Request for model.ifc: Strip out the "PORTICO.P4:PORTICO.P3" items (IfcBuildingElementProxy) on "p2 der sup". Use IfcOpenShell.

First a look at what the model holds.

```python
import ifcopenshell
import ifcopenshell.util.element

model = ifcopenshell.open("model.ifc")
print(model.schema)
storey = next(s for s in model.by_type("IfcBuildingStorey") if s.Name == "p2 der sup")
proxies = [e for e in ifcopenshell.util.element.get_decomposition(storey) if e.is_a("IfcBuildingElementProxy")]
seen = {}
for e in proxies:
    element_type = ifcopenshell.util.element.get_type(e)
    name = element_type.Name if element_type not in (None, e) else None
    seen[name] = seen.get(name, 0) + 1
for name, count in sorted(seen.items(), key=str):
    print(count, "x", name)
```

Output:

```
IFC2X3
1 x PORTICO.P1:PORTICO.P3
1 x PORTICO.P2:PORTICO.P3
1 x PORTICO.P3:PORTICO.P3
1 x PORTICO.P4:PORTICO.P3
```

```python
import ifcopenshell
import ifcopenshell.api.root
import ifcopenshell.util.element

model = ifcopenshell.open("model.ifc")

storey = next(s for s in model.by_type("IfcBuildingStorey") if s.Name == "p2 der sup")
proxies = [e for e in ifcopenshell.util.element.get_decomposition(storey) if e.is_a("IfcBuildingElementProxy")]
targets = [e for e in proxies if (t := ifcopenshell.util.element.get_type(e)) not in (None, e) and t.Name == "PORTICO.P4:PORTICO.P3"]

for e in targets:
    ifcopenshell.api.root.remove_product(model, product=e)
print(len(targets), "removed")

model.write("model_rev.ifc")
```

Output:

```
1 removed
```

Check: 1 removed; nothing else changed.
